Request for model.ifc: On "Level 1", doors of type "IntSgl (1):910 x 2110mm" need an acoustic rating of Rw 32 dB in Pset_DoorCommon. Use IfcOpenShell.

First a look at what the model holds.

```python
import ifcopenshell
import ifcopenshell.util.element

model = ifcopenshell.open("model.ifc")
print(model.schema)
storey = next(s for s in model.by_type("IfcBuildingStorey") if s.Name == "Level 1")
doors = [e for e in ifcopenshell.util.element.get_decomposition(storey) if e.is_a("IfcDoor")]
seen = {}
for e in doors:
    element_type = ifcopenshell.util.element.get_type(e)
    key = (element_type.Name if element_type != e and element_type else None, ifcopenshell.util.element.get_pset(e, "Pset_DoorCommon", "AcousticRating"))
    seen[key] = seen.get(key, 0) + 1
for (name, value), count in sorted(seen.items(), key=str):
    print(count, "x", name, "|", value)
```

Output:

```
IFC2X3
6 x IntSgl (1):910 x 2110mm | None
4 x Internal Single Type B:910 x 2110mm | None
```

```python
import ifcopenshell
import ifcopenshell.api.pset
import ifcopenshell.util.element

model = ifcopenshell.open("model.ifc")

storey = next(s for s in model.by_type("IfcBuildingStorey") if s.Name == "Level 1")
doors = [e for e in ifcopenshell.util.element.get_decomposition(storey) if e.is_a("IfcDoor")]

count = 0
for e in doors:
    element_type = ifcopenshell.util.element.get_type(e)
    if element_type in (None, e) or element_type.Name != "IntSgl (1):910 x 2110mm":
        continue
    # add_pset returns the element's existing set when there is one.
    pset = ifcopenshell.api.pset.add_pset(model, product=e, name="Pset_DoorCommon")
    ifcopenshell.api.pset.edit_pset(model, pset=pset, properties={"AcousticRating": "Rw 32 dB"})
    count += 1

print(count, "doors updated")

model.write("model-out.ifc")
```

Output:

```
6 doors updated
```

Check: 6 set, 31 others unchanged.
